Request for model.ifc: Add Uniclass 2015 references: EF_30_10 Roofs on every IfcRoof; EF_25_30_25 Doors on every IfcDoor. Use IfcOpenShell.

First a look at what the model holds.

```python
import ifcopenshell

model = ifcopenshell.open("model.ifc")
print(model.schema)
print("classifications:", [c.Name for c in model.by_type("IfcClassification")])
for ifc_class in ("IfcDoor", "IfcRoof", "IfcStair", "IfcWall", "IfcWindow"):
    print(ifc_class, len(model.by_type(ifc_class)))
```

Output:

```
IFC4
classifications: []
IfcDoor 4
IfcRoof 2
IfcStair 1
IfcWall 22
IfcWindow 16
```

```python
import ifcopenshell
import ifcopenshell.api.classification

model = ifcopenshell.open("model.ifc")

system = ifcopenshell.api.classification.add_classification(model, classification="Uniclass 2015")

codes = {
    "IfcRoof": ("EF_30_10", "Roofs"),
    "IfcDoor": ("EF_25_30_25", "Doors"),
}
for ifc_class, (code, name) in codes.items():
    products = model.by_type(ifc_class)
    ifcopenshell.api.classification.add_reference(
        model, products=products, classification=system, identification=code, name=name
    )
    print(code, len(products))

model.write("model_rev.ifc")
```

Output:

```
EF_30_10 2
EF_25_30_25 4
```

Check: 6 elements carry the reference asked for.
